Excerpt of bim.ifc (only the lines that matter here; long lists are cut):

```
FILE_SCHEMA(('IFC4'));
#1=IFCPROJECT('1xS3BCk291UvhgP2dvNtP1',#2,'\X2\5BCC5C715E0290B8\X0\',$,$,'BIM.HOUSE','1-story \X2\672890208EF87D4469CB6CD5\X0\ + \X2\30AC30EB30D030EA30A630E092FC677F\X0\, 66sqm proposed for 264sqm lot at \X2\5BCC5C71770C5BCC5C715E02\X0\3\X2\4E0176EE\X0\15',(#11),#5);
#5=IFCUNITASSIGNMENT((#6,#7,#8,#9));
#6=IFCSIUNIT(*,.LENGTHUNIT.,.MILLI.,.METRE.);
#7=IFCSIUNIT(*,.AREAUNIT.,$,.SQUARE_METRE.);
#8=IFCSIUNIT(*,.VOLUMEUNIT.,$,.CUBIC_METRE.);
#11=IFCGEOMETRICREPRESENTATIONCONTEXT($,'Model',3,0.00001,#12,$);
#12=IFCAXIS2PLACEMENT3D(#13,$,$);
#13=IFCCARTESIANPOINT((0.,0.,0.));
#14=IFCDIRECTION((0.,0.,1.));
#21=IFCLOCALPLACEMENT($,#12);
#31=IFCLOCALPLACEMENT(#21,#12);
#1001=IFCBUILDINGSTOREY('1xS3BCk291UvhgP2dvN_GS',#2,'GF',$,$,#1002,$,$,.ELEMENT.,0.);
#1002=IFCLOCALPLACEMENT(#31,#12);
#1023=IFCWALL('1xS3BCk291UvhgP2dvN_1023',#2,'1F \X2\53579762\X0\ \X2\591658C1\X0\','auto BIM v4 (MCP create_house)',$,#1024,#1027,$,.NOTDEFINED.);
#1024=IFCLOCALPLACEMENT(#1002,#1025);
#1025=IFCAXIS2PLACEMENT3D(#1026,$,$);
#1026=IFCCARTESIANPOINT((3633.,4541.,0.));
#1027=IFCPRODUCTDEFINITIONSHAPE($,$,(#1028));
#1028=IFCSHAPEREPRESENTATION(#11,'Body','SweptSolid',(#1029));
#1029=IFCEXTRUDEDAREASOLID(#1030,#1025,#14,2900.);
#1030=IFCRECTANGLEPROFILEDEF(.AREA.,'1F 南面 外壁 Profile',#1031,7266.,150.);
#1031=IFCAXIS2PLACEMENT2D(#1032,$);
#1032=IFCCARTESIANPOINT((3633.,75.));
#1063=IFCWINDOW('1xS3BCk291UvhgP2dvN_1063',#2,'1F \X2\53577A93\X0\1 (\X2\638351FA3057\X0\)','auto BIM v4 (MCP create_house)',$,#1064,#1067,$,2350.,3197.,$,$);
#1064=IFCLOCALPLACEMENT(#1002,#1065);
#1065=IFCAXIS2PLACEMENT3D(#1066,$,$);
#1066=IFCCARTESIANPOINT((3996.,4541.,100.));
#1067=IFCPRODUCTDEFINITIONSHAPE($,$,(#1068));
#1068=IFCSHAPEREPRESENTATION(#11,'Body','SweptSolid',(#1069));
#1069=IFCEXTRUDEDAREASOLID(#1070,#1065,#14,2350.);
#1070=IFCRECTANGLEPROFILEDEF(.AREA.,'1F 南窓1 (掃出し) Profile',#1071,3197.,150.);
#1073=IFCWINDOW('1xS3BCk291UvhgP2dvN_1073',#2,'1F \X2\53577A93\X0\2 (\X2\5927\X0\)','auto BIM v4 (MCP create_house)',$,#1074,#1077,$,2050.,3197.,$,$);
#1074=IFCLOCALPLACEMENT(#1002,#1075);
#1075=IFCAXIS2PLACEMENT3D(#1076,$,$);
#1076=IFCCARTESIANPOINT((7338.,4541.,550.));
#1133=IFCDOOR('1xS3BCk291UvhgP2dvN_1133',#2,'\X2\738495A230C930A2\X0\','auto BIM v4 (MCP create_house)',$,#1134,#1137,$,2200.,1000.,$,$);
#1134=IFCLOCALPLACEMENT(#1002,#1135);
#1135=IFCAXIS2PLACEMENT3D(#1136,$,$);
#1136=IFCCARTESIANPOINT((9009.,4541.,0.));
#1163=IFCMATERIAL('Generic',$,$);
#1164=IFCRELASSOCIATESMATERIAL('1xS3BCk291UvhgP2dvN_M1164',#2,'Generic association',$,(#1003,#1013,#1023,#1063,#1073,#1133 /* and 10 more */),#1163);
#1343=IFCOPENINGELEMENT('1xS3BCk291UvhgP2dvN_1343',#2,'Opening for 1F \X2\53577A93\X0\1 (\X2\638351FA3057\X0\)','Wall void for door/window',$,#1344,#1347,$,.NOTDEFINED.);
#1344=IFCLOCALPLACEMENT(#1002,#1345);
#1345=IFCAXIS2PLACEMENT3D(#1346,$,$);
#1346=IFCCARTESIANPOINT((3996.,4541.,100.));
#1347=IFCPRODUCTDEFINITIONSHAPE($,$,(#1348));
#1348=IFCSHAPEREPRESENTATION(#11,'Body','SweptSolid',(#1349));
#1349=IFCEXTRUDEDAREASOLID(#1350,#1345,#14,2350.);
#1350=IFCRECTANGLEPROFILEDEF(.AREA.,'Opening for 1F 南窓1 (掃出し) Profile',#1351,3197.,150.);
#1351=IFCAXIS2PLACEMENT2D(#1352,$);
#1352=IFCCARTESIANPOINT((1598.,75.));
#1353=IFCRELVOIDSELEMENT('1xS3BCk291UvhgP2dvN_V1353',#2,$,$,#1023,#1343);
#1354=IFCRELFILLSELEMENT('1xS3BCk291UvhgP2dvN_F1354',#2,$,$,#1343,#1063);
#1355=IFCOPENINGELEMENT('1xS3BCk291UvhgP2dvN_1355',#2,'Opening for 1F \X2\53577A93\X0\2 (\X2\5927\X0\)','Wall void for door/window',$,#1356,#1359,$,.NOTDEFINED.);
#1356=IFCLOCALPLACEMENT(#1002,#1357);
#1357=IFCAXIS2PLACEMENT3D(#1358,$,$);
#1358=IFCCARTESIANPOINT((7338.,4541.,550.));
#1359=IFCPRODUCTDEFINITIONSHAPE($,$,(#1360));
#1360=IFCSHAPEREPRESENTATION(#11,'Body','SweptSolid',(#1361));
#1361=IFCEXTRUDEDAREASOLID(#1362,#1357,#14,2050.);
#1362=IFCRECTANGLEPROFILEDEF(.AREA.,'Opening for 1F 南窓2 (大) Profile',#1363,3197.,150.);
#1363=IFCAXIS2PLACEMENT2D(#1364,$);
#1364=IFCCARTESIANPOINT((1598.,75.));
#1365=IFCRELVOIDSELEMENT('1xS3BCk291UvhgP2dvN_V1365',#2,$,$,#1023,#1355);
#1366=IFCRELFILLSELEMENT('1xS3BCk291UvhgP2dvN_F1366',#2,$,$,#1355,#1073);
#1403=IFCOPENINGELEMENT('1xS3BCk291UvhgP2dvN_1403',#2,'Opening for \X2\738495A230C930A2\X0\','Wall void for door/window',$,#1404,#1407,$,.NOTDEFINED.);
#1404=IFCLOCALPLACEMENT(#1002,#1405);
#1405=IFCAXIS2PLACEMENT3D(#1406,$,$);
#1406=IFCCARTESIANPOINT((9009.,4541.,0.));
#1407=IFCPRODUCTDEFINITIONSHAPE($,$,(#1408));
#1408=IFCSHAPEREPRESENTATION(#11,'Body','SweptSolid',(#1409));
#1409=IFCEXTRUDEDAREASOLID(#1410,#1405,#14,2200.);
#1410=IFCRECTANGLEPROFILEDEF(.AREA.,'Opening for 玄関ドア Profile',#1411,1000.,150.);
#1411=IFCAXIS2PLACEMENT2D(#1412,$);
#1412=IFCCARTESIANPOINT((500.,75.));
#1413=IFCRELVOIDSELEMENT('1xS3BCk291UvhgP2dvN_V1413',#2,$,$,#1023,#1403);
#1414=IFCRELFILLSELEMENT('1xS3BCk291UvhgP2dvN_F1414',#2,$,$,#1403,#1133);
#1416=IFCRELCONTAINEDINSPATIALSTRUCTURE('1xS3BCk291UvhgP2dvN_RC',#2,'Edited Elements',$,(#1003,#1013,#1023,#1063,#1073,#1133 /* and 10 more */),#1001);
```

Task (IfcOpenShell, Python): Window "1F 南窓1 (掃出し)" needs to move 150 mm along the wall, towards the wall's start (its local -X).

```python
import ifcopenshell
import ifcopenshell.api.geometry
import ifcopenshell.util.placement

model = ifcopenshell.open("bim.ifc")

window = model.by_guid("1xS3BCk291UvhgP2dvN_1063")
opening = window.FillsVoids[0].RelatingOpeningElement
wall = opening.VoidsElements[0].RelatingBuildingElement

wall_matrix = ifcopenshell.util.placement.get_local_placement(wall.ObjectPlacement)
shift = wall_matrix[:3, 0] * -150.0
before = ifcopenshell.util.placement.get_local_placement(window.ObjectPlacement)[:3, 3].copy()

# The window is not placed relative to its opening, so move both.
for product in (opening, window):
    matrix = ifcopenshell.util.placement.get_local_placement(product.ObjectPlacement)
    matrix[:3, 3] += shift
    ifcopenshell.api.geometry.edit_object_placement(model, product=product, matrix=matrix, is_si=False)

after = ifcopenshell.util.placement.get_local_placement(window.ObjectPlacement)[:3, 3]
print("window moved by", (after - before).round(3) + 0.0)

model.write("bim_edited.ifc")
```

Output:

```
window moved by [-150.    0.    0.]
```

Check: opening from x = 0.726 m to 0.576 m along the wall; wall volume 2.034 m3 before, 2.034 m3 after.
